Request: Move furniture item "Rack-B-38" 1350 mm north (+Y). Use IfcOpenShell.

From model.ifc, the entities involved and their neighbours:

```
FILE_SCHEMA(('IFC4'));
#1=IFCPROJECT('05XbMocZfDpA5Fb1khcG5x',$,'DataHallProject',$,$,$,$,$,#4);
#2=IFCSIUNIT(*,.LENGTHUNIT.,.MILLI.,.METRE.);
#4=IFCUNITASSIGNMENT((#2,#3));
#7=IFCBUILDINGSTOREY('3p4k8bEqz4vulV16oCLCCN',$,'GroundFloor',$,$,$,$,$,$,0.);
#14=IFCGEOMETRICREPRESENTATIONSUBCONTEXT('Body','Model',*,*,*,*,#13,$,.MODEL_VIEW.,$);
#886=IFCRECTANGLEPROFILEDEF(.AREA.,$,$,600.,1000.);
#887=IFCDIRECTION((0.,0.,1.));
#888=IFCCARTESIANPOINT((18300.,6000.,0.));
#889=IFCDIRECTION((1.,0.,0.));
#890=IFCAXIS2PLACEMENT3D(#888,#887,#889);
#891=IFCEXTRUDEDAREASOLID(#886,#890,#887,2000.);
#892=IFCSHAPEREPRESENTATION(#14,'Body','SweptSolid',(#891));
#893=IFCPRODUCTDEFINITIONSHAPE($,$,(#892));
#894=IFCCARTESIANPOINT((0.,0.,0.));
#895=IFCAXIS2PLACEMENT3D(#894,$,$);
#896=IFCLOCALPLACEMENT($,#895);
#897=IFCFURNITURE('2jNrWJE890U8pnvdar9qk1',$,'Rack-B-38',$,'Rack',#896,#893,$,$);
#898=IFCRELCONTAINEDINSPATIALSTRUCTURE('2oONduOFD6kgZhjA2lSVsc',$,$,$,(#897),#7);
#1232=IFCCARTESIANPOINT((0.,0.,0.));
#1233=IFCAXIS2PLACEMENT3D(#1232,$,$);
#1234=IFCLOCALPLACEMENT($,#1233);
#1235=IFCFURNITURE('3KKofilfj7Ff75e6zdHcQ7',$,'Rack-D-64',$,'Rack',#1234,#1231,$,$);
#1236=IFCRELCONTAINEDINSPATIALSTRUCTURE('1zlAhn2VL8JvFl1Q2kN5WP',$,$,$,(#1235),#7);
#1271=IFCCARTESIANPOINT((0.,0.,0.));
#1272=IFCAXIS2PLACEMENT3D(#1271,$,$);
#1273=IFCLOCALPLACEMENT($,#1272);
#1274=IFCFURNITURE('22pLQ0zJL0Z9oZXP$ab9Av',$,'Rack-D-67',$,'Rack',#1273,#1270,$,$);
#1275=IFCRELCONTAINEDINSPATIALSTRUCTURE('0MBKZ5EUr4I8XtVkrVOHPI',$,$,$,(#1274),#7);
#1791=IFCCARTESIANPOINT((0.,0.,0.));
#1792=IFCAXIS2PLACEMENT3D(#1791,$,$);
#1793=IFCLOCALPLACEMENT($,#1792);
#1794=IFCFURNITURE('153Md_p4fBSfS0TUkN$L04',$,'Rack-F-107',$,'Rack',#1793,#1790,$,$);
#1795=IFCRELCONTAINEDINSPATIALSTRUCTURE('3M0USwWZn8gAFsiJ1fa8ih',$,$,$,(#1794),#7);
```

```python
import ifcopenshell
import ifcopenshell.api.geometry
import ifcopenshell.util.placement

model = ifcopenshell.open("model.ifc")

item = model.by_guid("2jNrWJE890U8pnvdar9qk1")
matrix = ifcopenshell.util.placement.get_local_placement(item.ObjectPlacement)
matrix[1, 3] += 1350.0
ifcopenshell.api.geometry.edit_object_placement(model, product=item, matrix=matrix, is_si=False)

print(ifcopenshell.util.placement.get_local_placement(item.ObjectPlacement).round(3) + 0.0)

model.write("model_edited.ifc")
```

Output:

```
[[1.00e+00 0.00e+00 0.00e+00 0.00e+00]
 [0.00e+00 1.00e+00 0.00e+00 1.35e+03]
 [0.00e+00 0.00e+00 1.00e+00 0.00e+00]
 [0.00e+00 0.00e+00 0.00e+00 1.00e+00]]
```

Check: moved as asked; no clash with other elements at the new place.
